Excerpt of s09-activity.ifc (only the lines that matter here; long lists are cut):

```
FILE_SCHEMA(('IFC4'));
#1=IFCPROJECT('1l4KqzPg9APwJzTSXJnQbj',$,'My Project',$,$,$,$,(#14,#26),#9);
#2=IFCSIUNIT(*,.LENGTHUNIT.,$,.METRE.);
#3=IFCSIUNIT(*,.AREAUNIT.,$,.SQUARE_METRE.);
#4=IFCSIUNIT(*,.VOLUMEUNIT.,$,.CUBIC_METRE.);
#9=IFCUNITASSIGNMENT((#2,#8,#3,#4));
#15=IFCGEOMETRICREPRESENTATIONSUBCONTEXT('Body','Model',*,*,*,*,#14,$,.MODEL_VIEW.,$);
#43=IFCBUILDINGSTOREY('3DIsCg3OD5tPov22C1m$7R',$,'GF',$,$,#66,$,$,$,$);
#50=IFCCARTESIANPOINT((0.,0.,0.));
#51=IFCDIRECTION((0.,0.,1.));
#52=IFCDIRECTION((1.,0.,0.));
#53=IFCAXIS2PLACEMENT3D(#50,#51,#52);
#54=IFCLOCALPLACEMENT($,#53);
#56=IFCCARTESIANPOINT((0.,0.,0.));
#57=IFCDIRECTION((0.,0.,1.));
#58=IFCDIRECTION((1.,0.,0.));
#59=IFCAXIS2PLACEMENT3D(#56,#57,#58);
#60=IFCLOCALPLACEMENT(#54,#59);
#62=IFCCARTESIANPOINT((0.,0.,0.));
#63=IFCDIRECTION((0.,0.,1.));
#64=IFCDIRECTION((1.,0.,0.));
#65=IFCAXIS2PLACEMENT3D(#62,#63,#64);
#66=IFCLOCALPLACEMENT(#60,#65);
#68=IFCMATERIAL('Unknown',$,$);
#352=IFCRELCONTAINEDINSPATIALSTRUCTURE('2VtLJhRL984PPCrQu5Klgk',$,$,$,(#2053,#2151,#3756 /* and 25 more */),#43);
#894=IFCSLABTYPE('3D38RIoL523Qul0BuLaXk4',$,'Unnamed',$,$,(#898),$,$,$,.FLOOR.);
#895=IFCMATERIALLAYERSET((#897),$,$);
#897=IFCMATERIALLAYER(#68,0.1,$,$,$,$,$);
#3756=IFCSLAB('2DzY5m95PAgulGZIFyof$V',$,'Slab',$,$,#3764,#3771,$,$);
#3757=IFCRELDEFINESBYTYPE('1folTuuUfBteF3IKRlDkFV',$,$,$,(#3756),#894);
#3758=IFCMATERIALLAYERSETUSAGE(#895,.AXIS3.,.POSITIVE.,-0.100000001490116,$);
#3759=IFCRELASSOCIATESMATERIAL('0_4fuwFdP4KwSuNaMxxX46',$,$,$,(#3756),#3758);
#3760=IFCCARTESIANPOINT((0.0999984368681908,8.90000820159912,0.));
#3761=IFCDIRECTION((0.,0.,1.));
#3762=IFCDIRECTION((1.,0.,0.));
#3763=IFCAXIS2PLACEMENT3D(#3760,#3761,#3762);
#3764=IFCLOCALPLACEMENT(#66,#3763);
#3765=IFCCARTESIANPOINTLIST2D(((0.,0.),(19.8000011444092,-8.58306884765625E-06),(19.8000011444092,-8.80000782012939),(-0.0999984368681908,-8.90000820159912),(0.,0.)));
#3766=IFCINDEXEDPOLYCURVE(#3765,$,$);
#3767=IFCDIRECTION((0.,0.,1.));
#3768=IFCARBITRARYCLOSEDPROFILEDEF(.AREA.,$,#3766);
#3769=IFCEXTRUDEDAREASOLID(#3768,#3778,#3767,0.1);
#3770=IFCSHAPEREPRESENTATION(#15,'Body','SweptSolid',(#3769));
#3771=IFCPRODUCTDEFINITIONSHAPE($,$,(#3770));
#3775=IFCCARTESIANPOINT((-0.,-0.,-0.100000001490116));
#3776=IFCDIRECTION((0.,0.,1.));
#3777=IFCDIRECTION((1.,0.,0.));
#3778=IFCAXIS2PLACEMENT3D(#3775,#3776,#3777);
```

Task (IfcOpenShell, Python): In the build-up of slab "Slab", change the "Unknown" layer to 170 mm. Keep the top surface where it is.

```python
import ifcopenshell
import ifcopenshell.util.element
import ifcopenshell.util.representation
import ifcopenshell.util.unit

model = ifcopenshell.open("s09-activity.ifc")
unit_scale = ifcopenshell.util.unit.calculate_unit_scale(model)

layer_set = model.by_id(895)
layer = next(l for l in layer_set.MaterialLayers if l.Material and l.Material.Name == "Unknown")
change = 0.17 / unit_scale - layer.LayerThickness
layer.LayerThickness += change

# Geometry does not follow the layer set by itself.
slabs = [e for e in ifcopenshell.util.element.get_elements_by_material(model, layer_set) if e.is_a("IfcSlab")]
for slab in sorted(slabs, key=lambda e: e.id()):
    body = ifcopenshell.util.representation.get_representation(slab, "Model", "Body")
    solid = body.Items[0]
    old_depth = solid.Depth
    solid.Depth += change
    # Extruded upwards: lower the start of the extrusion so the top stays.
    x, y, z = solid.Position.Location.Coordinates
    solid.Position.Location = model.createIfcCartesianPoint((x, y, z - change))
    print(slab.id(), f"{old_depth:g} -> {solid.Depth:g}")

# The layers are counted up from the underside, which has moved.
for usage in {ifcopenshell.util.element.get_material(slab) for slab in slabs}:
    usage.OffsetFromReferenceLine -= change

model.write("s09-activity-out.ifc")
```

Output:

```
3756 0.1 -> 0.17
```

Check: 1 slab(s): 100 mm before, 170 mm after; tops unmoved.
